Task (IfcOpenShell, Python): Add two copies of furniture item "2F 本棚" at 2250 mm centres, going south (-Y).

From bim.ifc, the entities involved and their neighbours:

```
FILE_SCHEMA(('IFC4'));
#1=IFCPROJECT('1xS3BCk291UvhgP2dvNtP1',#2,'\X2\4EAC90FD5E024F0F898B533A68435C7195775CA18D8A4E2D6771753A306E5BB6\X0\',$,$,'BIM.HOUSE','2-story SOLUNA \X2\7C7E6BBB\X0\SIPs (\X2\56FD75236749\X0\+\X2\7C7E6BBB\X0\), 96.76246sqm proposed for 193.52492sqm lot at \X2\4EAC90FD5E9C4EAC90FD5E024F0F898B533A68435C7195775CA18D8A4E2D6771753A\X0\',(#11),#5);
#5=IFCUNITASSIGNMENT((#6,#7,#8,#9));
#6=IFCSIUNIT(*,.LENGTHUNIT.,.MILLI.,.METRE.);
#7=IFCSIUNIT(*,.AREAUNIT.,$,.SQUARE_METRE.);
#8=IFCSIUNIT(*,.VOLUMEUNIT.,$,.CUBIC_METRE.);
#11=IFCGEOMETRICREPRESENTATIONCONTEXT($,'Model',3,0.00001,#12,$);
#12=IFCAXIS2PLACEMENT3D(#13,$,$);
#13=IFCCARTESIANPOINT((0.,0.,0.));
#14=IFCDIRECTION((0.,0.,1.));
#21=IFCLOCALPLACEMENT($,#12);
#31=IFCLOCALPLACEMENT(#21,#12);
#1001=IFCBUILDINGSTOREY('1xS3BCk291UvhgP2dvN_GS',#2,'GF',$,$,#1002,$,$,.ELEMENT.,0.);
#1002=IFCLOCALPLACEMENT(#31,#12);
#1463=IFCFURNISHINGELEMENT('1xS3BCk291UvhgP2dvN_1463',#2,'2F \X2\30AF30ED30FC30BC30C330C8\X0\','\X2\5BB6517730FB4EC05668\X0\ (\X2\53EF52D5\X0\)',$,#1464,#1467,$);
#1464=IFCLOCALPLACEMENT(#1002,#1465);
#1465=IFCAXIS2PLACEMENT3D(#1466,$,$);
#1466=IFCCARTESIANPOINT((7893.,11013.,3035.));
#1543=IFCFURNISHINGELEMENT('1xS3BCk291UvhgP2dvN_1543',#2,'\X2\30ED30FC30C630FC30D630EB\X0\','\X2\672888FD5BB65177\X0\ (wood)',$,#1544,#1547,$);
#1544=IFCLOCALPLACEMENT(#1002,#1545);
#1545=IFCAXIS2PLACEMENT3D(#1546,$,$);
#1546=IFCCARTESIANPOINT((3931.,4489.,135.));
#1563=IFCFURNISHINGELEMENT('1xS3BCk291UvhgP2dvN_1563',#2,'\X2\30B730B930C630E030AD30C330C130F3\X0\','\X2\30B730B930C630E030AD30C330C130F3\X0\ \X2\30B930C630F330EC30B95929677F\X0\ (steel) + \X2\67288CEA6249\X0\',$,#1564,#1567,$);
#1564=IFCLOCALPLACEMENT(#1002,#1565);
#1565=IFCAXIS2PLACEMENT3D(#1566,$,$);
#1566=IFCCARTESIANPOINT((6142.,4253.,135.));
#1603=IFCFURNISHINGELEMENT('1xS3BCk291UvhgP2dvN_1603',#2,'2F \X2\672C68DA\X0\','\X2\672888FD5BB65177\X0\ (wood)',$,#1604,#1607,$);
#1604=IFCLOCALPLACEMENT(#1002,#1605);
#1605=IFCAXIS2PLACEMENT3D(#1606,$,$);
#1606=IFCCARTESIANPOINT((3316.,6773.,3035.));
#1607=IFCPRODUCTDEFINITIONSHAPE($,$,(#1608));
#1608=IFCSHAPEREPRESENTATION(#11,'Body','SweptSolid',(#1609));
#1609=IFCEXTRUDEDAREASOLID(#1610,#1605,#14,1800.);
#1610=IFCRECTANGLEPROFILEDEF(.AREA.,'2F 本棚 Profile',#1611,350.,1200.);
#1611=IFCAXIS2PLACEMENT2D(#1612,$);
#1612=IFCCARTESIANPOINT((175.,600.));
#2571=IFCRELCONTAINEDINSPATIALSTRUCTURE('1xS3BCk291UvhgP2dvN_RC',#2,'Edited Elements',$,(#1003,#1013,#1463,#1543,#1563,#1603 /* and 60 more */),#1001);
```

```python
import numpy as np
import ifcopenshell
import ifcopenshell.api.geometry
import ifcopenshell.api.root
import ifcopenshell.util.element
import ifcopenshell.util.placement

model = ifcopenshell.open("bim.ifc")


def reuse_history(source, copy):
    """copy_class also copies each property set's owner history, people and application; keep the originals."""
    for rel in copy.IsDefinedBy:
        if rel.is_a("IfcRelDefinesByProperties") and (history := rel.RelatingPropertyDefinition.OwnerHistory):
            rel.RelatingPropertyDefinition.OwnerHistory = source.OwnerHistory
            ifcopenshell.util.element.remove_deep2(model, history)


source = model.by_guid("1xS3BCk291UvhgP2dvN_1603")
base = ifcopenshell.util.placement.get_local_placement(source.ObjectPlacement)
step = np.array([0.0, -1.0, 0.0]) * 2250.0

for i in range(1, 3):
    copy = ifcopenshell.api.root.copy_class(model, product=source)
    copy.Representation = ifcopenshell.util.element.copy_deep(
        model, source.Representation, exclude=["IfcGeometricRepresentationContext", "IfcRepresentationMap"]
    )
    reuse_history(source, copy)
    matrix = base.copy()
    matrix[:3, 3] += i * step
    print("added at", matrix[:3, 3].round(3) + 0.0)
    ifcopenshell.api.geometry.edit_object_placement(model, product=copy, matrix=matrix, is_si=False)

model.write("bim_v2.ifc")
```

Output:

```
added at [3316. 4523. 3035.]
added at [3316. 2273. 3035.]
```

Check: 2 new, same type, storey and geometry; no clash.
